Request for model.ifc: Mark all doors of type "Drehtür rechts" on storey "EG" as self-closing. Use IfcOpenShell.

First a look at what the model holds.

```python
import ifcopenshell
import ifcopenshell.util.element

model = ifcopenshell.open("model.ifc")
print(model.schema)
storey = next(s for s in model.by_type("IfcBuildingStorey") if s.Name == "EG")
doors = [e for e in ifcopenshell.util.element.get_decomposition(storey) if e.is_a("IfcDoor")]
seen = {}
for e in doors:
    element_type = ifcopenshell.util.element.get_type(e)
    key = (element_type.Name if element_type != e and element_type else None, ifcopenshell.util.element.get_pset(e, "Pset_DoorCommon", "SelfClosing"))
    seen[key] = seen.get(key, 0) + 1
for (name, value), count in sorted(seen.items(), key=str):
    print(count, "x", name, "|", value)
```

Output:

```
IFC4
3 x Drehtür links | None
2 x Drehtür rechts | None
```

```python
import ifcopenshell
import ifcopenshell.api.pset
import ifcopenshell.util.element

model = ifcopenshell.open("model.ifc")

storey = next(s for s in model.by_type("IfcBuildingStorey") if s.Name == "EG")
doors = [e for e in ifcopenshell.util.element.get_decomposition(storey) if e.is_a("IfcDoor")]

count = 0
for e in doors:
    element_type = ifcopenshell.util.element.get_type(e)
    if element_type in (None, e) or element_type.Name != "Drehtür rechts":
        continue
    # add_pset returns the element's existing set when there is one.
    pset = ifcopenshell.api.pset.add_pset(model, product=e, name="Pset_DoorCommon")
    ifcopenshell.api.pset.edit_pset(model, pset=pset, properties={"SelfClosing": True})
    count += 1

print(count, "doors updated")

model.write("model_rev.ifc")
```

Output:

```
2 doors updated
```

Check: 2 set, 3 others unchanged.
